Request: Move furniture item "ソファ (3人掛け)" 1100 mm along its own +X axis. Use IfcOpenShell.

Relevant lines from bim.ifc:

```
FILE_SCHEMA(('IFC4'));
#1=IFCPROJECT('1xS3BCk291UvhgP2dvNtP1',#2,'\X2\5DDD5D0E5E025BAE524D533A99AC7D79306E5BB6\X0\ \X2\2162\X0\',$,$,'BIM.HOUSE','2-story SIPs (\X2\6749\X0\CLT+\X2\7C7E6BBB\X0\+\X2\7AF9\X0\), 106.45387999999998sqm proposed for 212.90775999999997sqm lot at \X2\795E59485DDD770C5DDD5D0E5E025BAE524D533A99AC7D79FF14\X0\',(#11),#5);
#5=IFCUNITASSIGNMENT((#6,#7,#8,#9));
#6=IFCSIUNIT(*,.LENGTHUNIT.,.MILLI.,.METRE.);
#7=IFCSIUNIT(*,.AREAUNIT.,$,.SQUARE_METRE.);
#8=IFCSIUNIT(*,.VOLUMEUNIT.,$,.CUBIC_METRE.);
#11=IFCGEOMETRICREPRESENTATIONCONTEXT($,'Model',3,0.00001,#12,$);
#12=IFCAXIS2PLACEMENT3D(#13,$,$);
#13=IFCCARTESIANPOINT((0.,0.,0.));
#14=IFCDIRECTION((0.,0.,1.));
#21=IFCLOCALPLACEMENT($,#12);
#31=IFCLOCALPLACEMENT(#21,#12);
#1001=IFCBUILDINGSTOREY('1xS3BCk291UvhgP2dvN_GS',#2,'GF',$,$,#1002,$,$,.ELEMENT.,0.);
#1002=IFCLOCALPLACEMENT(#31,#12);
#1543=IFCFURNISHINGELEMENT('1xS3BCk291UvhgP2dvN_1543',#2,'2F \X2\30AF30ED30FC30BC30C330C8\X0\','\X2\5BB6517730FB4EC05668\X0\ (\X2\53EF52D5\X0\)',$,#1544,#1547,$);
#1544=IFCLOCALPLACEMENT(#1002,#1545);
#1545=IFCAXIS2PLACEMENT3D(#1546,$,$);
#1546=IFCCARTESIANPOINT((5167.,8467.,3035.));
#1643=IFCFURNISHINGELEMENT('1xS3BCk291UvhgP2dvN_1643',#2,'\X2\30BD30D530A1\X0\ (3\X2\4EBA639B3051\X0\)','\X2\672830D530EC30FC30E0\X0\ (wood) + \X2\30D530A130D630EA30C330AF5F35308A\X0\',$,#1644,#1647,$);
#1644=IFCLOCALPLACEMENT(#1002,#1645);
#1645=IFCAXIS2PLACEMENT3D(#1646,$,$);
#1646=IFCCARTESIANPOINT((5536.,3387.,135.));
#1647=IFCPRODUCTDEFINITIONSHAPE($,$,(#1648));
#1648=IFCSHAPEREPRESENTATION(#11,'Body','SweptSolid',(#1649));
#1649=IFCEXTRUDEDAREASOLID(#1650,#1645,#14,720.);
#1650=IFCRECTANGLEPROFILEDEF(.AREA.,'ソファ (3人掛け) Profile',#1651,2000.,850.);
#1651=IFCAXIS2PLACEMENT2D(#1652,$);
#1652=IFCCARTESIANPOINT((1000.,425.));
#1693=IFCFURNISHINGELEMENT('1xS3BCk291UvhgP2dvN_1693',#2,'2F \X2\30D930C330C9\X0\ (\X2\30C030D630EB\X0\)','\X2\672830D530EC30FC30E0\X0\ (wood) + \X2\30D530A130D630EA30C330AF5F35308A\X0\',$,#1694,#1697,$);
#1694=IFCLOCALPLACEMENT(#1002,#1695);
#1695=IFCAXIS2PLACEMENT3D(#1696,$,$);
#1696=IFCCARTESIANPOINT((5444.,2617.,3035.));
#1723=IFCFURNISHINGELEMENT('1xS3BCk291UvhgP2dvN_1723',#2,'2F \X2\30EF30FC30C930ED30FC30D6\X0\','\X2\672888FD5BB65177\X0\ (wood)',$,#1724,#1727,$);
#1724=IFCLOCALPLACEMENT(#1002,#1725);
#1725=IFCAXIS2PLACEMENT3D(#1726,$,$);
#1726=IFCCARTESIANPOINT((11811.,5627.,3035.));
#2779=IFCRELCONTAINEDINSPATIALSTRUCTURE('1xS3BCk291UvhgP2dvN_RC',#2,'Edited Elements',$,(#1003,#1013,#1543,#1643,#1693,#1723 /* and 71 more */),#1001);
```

```python
import ifcopenshell
import ifcopenshell.api.geometry
import ifcopenshell.util.placement
import ifcopenshell.util.unit

model = ifcopenshell.open("bim.ifc")
unit_scale = ifcopenshell.util.unit.calculate_unit_scale(model)

item = model.by_guid("1xS3BCk291UvhgP2dvN_1643")
matrix = ifcopenshell.util.placement.get_local_placement(item.ObjectPlacement)
matrix[:3, 3] += matrix[:3, 0] * 1.1 / unit_scale
ifcopenshell.api.geometry.edit_object_placement(model, product=item, matrix=matrix, is_si=False)

print(ifcopenshell.util.placement.get_local_placement(item.ObjectPlacement).round(3) + 0.0)

model.write("bim-out.ifc")
```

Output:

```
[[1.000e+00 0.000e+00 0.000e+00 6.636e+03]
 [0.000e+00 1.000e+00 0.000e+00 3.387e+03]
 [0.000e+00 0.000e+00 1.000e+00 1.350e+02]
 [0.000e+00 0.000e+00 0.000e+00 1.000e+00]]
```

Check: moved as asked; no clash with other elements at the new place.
